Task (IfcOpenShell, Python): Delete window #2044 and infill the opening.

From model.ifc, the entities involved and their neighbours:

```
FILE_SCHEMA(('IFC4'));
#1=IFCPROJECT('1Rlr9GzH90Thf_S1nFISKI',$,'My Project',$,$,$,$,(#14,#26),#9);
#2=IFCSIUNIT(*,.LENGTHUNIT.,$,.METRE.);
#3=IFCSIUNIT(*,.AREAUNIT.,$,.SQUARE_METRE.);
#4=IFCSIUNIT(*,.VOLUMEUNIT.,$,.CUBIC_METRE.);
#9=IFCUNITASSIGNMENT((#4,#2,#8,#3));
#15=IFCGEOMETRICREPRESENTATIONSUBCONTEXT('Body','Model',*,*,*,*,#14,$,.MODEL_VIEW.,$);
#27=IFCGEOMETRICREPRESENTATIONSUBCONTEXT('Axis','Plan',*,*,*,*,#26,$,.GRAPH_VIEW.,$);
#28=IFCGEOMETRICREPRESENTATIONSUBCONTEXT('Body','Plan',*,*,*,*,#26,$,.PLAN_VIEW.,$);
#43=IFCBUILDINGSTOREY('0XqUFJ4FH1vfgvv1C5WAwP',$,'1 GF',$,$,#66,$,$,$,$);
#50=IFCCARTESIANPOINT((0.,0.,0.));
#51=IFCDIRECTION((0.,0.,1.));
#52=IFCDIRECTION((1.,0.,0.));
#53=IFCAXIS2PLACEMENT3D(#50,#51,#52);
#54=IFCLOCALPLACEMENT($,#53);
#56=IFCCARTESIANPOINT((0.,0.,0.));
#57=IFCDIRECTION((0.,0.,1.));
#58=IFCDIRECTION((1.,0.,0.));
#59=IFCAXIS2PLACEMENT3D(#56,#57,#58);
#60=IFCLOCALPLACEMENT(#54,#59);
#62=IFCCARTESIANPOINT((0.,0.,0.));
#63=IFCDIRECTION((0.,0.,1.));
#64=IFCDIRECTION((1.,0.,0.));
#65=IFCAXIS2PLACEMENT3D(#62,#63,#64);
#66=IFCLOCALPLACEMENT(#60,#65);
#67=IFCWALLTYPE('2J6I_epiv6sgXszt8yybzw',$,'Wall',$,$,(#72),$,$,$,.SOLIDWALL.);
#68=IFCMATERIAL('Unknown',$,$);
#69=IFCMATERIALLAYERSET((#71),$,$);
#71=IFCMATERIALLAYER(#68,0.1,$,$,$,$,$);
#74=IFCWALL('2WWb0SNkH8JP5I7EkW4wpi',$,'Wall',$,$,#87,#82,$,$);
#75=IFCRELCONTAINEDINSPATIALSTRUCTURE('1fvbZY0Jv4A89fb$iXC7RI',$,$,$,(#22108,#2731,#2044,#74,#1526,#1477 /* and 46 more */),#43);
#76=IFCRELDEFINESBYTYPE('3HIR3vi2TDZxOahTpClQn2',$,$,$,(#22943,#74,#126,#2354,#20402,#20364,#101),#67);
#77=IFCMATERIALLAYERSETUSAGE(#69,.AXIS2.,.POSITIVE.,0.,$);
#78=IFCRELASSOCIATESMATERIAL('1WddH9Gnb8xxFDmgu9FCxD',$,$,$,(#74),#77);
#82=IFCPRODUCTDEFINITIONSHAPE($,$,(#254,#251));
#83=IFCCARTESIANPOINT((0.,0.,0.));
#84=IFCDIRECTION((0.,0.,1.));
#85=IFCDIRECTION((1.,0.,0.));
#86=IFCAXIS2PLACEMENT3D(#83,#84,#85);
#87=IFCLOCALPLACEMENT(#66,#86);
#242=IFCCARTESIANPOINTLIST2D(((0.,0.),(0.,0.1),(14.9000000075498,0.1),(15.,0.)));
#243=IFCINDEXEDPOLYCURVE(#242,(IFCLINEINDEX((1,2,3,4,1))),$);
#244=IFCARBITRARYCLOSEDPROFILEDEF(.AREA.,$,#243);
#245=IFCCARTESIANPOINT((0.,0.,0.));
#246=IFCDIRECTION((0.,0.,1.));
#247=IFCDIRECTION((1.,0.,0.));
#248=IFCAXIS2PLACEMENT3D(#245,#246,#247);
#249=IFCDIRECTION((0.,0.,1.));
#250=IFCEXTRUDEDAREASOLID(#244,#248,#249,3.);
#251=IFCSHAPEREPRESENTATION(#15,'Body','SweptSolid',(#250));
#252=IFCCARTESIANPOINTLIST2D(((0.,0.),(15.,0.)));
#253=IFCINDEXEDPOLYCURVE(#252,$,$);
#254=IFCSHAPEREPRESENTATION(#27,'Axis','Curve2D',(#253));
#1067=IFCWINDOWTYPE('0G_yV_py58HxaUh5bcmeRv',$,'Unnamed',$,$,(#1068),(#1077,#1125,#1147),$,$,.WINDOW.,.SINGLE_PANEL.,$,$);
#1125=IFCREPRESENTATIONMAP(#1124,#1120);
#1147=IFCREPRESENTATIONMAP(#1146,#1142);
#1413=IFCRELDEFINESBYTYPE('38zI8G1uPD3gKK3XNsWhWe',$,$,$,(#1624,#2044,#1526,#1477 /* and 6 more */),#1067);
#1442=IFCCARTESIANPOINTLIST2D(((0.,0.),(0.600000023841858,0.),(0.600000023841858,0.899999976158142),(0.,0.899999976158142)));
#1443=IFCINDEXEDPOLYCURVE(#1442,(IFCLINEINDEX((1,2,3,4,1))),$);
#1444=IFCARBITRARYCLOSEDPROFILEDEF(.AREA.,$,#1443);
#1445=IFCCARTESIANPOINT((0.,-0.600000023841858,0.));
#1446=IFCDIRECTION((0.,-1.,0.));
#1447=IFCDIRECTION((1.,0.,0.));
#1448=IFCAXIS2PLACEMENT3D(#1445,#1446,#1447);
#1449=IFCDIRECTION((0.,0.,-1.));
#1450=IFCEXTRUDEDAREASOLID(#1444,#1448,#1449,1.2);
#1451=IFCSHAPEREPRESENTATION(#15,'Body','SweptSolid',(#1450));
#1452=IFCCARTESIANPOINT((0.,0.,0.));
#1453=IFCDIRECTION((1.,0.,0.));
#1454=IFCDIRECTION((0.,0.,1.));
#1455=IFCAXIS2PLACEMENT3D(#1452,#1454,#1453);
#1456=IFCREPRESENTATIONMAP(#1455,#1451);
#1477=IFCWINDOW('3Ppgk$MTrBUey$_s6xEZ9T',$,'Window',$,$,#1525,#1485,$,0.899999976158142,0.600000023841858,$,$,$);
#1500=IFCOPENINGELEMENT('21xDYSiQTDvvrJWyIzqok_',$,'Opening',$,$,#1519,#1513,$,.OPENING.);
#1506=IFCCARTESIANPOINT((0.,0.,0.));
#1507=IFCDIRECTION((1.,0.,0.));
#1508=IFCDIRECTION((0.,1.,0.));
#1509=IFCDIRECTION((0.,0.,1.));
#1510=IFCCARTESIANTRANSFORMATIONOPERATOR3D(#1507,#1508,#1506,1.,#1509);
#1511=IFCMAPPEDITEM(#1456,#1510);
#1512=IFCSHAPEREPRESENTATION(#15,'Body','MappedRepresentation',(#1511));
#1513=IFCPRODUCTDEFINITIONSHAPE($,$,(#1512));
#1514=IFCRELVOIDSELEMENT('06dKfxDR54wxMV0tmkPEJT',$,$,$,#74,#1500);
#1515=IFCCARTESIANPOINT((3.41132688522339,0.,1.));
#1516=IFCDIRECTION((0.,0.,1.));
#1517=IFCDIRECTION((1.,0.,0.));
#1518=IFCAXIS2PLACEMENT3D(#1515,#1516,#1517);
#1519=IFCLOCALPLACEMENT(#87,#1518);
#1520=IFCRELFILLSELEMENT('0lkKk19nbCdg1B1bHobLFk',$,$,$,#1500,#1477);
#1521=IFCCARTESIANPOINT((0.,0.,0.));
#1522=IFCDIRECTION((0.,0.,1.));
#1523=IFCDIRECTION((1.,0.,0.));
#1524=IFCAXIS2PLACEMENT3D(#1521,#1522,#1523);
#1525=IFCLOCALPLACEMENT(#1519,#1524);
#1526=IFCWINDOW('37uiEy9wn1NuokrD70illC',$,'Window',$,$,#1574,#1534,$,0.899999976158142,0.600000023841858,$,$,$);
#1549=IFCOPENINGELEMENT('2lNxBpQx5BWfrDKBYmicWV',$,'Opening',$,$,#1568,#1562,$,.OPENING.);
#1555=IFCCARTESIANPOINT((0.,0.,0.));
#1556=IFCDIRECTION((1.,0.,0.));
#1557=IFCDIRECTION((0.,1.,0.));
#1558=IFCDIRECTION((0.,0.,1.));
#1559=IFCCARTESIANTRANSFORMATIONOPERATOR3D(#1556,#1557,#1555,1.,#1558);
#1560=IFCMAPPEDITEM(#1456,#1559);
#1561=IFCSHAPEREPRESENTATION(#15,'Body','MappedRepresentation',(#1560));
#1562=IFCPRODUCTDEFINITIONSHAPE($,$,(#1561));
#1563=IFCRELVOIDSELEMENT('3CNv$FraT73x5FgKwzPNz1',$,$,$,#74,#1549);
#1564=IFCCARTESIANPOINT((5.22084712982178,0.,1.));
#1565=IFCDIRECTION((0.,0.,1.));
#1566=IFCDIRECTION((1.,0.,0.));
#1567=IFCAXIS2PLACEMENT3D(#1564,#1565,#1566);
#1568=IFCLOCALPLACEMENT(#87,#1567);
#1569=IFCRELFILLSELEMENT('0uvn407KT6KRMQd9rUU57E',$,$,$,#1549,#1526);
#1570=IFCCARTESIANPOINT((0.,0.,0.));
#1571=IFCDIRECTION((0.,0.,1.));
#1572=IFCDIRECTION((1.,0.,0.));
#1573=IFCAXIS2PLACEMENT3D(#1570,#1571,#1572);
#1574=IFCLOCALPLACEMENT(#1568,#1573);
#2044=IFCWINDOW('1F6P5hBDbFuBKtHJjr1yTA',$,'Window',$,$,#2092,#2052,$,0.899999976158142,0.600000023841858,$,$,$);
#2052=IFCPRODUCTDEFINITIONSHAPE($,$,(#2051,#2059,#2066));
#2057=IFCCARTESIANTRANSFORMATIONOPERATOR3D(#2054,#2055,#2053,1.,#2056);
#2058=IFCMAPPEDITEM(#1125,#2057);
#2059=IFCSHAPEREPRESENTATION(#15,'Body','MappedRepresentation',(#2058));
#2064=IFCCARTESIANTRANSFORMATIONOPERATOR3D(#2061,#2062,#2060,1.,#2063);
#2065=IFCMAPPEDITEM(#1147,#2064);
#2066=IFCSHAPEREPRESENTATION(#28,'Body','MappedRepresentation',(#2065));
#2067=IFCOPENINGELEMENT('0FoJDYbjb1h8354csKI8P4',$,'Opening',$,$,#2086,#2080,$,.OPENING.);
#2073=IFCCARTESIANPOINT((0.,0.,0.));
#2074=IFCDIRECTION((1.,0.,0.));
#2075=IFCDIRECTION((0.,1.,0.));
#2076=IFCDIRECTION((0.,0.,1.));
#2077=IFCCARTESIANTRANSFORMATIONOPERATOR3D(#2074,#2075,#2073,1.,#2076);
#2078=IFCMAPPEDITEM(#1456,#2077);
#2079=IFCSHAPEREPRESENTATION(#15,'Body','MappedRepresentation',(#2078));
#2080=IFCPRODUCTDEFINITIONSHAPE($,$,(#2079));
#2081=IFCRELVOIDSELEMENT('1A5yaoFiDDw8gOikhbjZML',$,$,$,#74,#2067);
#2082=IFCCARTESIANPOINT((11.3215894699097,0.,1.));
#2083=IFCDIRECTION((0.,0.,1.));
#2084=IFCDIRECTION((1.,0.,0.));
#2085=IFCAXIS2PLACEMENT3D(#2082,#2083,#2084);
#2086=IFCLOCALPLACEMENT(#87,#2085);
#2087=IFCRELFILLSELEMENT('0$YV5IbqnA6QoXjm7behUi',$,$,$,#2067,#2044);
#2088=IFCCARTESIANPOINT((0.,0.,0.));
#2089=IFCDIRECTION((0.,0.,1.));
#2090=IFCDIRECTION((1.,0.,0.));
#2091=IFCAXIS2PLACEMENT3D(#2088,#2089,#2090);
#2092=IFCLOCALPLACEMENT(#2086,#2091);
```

```python
import ifcopenshell
import ifcopenshell.api.feature
import ifcopenshell.api.root
import ifcopenshell.geom
import ifcopenshell.util.shape

model = ifcopenshell.open("model.ifc")
settings = ifcopenshell.geom.settings()


def volume(element):
    """Net volume in cubic metres, openings subtracted."""
    shape = ifcopenshell.geom.create_shape(settings, element)
    return ifcopenshell.util.shape.get_volume(shape.geometry)


window = model.by_id(2044)
opening = window.FillsVoids[0].RelatingOpeningElement
wall = opening.VoidsElements[0].RelatingBuildingElement
before = volume(wall)

ifcopenshell.api.root.remove_product(model, product=window)
ifcopenshell.api.feature.remove_feature(model, feature=opening)

after = volume(wall)

print(f"wall volume {before:.3f} -> {after:.3f} m3")

model.write("model_v2.ifc")
```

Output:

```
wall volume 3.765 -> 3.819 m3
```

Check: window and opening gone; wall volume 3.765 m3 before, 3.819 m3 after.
